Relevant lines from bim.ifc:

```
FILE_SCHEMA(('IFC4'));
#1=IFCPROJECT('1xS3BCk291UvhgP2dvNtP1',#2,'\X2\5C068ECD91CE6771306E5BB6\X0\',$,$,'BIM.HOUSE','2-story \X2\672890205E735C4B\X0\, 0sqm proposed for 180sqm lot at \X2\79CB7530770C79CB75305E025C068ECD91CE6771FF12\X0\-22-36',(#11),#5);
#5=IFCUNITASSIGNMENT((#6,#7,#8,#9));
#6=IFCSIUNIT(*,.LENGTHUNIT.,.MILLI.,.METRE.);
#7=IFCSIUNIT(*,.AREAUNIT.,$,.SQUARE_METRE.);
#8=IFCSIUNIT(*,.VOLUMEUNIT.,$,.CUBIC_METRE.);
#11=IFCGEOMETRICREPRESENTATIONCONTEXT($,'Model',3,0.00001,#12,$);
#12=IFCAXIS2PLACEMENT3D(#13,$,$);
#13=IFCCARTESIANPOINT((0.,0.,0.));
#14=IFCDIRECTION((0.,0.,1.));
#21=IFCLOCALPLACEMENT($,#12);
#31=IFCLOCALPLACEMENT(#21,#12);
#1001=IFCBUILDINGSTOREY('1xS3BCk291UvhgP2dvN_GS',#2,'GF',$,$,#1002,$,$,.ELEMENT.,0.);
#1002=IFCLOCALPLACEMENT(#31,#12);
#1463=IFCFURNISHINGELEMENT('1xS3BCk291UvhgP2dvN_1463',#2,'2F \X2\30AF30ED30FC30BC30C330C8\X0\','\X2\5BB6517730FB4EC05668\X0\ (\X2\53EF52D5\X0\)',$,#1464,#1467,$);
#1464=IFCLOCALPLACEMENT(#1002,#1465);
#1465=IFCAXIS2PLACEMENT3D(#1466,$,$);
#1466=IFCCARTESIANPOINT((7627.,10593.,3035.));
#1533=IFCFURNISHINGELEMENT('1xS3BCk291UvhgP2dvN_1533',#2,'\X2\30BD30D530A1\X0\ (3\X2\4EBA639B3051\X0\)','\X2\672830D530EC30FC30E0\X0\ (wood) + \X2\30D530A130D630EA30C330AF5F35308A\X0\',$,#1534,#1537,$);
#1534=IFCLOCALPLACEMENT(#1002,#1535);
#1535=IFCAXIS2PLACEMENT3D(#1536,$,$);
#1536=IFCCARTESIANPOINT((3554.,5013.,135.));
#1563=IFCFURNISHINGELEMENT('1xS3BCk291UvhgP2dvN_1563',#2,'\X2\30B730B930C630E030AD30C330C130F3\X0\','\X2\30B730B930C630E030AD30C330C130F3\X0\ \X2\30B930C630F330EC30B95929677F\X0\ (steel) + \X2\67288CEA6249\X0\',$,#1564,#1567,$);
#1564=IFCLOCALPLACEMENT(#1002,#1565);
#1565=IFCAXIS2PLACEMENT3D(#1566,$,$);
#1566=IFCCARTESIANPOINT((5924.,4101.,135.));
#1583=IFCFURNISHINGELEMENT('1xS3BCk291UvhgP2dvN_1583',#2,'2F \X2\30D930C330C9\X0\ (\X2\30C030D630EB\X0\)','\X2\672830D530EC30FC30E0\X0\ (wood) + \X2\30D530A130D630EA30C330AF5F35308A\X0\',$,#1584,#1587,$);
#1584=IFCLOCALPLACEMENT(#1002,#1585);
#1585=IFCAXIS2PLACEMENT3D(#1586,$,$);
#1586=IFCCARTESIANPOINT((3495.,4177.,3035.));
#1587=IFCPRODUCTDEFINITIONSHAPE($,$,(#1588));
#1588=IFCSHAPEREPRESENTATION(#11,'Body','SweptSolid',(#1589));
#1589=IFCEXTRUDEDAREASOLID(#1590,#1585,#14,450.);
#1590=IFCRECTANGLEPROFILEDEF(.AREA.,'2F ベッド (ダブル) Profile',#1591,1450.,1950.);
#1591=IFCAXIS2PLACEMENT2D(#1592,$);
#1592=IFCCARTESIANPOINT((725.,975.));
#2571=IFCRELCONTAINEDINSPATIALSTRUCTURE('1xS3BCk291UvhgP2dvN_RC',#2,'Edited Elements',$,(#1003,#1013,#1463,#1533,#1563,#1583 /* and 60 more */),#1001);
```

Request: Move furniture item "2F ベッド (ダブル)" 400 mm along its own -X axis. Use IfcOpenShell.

```python
import ifcopenshell
import ifcopenshell.api.geometry
import ifcopenshell.util.placement
import ifcopenshell.util.unit

model = ifcopenshell.open("bim.ifc")
unit_scale = ifcopenshell.util.unit.calculate_unit_scale(model)

item = model.by_guid("1xS3BCk291UvhgP2dvN_1583")
matrix = ifcopenshell.util.placement.get_local_placement(item.ObjectPlacement)
matrix[:3, 3] -= matrix[:3, 0] * 0.4 / unit_scale
ifcopenshell.api.geometry.edit_object_placement(model, product=item, matrix=matrix, is_si=False)

print(ifcopenshell.util.placement.get_local_placement(item.ObjectPlacement).round(3) + 0.0)

model.write("bim_edited.ifc")
```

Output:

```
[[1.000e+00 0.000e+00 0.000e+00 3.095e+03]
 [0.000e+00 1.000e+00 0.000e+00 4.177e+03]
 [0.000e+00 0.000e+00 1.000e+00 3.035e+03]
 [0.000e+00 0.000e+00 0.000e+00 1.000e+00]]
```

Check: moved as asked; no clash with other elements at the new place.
